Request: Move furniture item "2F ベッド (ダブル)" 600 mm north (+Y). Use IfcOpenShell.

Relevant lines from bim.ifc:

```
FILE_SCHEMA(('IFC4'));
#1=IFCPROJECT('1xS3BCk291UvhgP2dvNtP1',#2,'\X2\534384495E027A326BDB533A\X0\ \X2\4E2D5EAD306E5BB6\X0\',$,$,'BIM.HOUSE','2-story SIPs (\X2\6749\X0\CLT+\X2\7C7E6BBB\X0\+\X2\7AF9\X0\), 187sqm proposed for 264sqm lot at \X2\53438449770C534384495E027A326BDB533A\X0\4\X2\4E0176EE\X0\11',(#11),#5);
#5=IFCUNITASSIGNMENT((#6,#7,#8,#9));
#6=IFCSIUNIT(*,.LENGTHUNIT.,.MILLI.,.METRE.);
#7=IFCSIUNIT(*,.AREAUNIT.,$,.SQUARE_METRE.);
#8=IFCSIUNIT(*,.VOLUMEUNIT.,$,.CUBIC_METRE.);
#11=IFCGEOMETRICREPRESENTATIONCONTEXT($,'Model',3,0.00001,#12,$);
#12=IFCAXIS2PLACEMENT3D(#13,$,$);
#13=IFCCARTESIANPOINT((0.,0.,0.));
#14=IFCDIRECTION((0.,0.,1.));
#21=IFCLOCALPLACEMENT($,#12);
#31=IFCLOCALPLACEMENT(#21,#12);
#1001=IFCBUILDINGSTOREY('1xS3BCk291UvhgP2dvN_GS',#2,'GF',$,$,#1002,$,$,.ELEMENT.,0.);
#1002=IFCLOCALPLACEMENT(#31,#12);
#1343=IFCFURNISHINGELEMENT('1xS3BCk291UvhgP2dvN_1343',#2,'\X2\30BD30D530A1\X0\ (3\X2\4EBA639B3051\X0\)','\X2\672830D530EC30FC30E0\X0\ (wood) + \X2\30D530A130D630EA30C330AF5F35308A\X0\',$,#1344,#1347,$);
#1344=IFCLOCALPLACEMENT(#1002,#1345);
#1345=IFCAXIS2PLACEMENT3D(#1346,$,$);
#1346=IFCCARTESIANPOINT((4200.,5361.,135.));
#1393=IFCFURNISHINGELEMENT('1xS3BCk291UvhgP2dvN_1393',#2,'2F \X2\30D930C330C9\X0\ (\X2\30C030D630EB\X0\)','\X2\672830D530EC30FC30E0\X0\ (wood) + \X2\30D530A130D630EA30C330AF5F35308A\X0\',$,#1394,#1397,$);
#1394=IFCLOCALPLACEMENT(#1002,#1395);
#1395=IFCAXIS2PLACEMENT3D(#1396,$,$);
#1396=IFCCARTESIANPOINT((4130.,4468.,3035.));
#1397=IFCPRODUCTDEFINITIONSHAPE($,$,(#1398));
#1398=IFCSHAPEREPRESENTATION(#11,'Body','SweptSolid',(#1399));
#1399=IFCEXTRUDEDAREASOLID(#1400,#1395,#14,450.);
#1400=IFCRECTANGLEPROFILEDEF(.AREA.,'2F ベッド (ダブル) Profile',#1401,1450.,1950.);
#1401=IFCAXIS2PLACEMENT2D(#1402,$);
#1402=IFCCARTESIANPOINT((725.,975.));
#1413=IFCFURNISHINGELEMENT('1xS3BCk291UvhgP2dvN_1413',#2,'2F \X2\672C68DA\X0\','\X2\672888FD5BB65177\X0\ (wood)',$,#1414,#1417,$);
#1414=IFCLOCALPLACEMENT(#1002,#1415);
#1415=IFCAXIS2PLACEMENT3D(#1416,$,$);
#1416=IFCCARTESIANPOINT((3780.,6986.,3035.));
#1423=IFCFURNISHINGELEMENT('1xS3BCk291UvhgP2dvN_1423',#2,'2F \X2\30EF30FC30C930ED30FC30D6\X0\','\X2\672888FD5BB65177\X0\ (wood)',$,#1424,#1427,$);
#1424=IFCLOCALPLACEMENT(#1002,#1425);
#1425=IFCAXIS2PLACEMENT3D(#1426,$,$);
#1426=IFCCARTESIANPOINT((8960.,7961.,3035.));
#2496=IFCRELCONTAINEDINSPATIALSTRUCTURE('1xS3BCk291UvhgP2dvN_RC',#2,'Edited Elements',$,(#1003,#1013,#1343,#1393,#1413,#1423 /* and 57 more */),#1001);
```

```python
import ifcopenshell
import ifcopenshell.api.geometry
import ifcopenshell.util.placement

model = ifcopenshell.open("bim.ifc")

item = model.by_guid("1xS3BCk291UvhgP2dvN_1393")
matrix = ifcopenshell.util.placement.get_local_placement(item.ObjectPlacement)
matrix[1, 3] += 600.0
ifcopenshell.api.geometry.edit_object_placement(model, product=item, matrix=matrix, is_si=False)

print(ifcopenshell.util.placement.get_local_placement(item.ObjectPlacement).round(3) + 0.0)

model.write("bim_edited.ifc")
```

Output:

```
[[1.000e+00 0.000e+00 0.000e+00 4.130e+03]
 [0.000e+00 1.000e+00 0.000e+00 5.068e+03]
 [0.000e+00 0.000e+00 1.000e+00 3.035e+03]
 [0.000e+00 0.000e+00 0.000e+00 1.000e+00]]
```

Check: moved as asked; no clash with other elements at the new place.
